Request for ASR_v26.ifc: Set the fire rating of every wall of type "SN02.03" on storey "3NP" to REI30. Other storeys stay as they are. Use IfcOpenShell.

First a look at what the model holds.

```python
import ifcopenshell
import ifcopenshell.util.element

model = ifcopenshell.open("ASR_v26.ifc")
print(model.schema)
storey = next(s for s in model.by_type("IfcBuildingStorey") if s.Name == "3NP")
walls = [e for e in ifcopenshell.util.element.get_decomposition(storey) if e.is_a("IfcWall")]
seen = {}
for e in walls:
    element_type = ifcopenshell.util.element.get_type(e)
    key = (element_type.Name if element_type != e and element_type else None, ifcopenshell.util.element.get_pset(e, "Pset_WallCommon", "FireRating"))
    seen[key] = seen.get(key, 0) + 1
for (name, value), count in sorted(seen.items(), key=str):
    print(count, "x", name, "|", value)
```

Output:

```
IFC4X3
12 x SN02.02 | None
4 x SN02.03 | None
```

```python
import ifcopenshell
import ifcopenshell.api.pset
import ifcopenshell.util.element

model = ifcopenshell.open("ASR_v26.ifc")

storey = next(s for s in model.by_type("IfcBuildingStorey") if s.Name == "3NP")
walls = [e for e in ifcopenshell.util.element.get_decomposition(storey) if e.is_a("IfcWall")]

count = 0
for e in walls:
    element_type = ifcopenshell.util.element.get_type(e)
    if element_type in (None, e) or element_type.Name != "SN02.03":
        continue
    # add_pset returns the element's existing set when there is one.
    pset = ifcopenshell.api.pset.add_pset(model, product=e, name="Pset_WallCommon")
    ifcopenshell.api.pset.edit_pset(model, pset=pset, properties={"FireRating": "REI30"})
    count += 1

print(count, "walls updated")

model.write("ASR_v26_rev.ifc")
```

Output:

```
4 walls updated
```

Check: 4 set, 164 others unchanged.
